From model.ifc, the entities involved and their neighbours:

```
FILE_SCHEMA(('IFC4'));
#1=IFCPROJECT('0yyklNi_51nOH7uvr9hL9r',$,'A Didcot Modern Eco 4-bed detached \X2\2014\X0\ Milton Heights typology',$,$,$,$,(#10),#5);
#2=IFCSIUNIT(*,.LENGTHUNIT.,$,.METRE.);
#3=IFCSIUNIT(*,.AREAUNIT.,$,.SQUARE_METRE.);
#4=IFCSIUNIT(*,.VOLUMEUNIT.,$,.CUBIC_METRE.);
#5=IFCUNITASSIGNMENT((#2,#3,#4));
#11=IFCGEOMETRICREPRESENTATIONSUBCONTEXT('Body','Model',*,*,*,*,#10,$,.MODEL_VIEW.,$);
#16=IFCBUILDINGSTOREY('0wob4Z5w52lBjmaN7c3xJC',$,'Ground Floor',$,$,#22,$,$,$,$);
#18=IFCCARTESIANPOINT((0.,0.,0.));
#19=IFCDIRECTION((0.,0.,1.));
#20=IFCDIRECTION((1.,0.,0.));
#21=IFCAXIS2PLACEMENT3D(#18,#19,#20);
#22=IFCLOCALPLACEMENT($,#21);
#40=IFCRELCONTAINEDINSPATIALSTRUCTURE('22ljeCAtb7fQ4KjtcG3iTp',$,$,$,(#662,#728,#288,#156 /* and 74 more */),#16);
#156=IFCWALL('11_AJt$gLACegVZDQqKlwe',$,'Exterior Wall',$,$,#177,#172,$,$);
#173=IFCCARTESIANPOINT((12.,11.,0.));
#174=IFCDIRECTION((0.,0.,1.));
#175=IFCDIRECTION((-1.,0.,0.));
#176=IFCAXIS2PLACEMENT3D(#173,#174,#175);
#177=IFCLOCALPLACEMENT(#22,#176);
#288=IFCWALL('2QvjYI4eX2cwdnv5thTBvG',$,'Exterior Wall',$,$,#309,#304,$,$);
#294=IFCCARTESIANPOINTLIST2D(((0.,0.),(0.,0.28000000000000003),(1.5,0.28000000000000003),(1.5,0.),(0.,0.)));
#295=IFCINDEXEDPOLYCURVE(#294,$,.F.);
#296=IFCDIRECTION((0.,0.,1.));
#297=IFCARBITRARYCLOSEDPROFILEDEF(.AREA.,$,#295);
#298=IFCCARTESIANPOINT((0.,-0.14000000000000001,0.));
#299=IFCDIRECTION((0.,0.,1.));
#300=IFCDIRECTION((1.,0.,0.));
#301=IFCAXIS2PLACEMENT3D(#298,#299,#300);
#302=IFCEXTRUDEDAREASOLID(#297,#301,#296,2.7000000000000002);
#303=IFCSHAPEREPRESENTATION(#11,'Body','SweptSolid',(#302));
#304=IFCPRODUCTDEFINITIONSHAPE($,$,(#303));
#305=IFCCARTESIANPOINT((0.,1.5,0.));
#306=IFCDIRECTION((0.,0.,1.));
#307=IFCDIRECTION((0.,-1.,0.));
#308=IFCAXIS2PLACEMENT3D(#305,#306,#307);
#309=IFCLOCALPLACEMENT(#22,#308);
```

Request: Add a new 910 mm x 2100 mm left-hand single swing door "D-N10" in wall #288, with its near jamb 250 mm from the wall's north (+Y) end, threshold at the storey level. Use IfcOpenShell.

```python
import numpy as np
import ifcopenshell
import ifcopenshell.api.feature
import ifcopenshell.api.geometry
import ifcopenshell.api.root
import ifcopenshell.api.spatial
import ifcopenshell.geom
import ifcopenshell.util.element
import ifcopenshell.util.placement
import ifcopenshell.util.representation
import ifcopenshell.util.shape
import ifcopenshell.util.unit

model = ifcopenshell.open("model.ifc")
unit_scale = ifcopenshell.util.unit.calculate_unit_scale(model)
settings = ifcopenshell.geom.settings()


def volume(element):
    """Net volume in cubic metres, openings subtracted."""
    shape = ifcopenshell.geom.create_shape(settings, element)
    return ifcopenshell.util.shape.get_volume(shape.geometry)


wall = model.by_id(288)
storey = ifcopenshell.util.element.get_container(wall, ifc_class="IfcBuildingStorey")
context = ifcopenshell.util.representation.get_context(model, "Model", "Body", "MODEL_VIEW")
before = volume(wall)

width, height, from_end, sill = 0.91, 2.1, 0.25, 0.0  # metres

# The wall runs along its own X axis, and the end named is its -X end.
wall_shape = ifcopenshell.geom.create_shape(settings, wall)
x, y, z = ifcopenshell.util.shape.get_vertices(wall_shape.geometry).T
start = x.min() + from_end
face, thickness = float(y.min()), float(y.max() - y.min())
wall_matrix = ifcopenshell.util.placement.get_local_placement(wall.ObjectPlacement)
level = ifcopenshell.util.placement.get_local_placement(storey.ObjectPlacement)[2, 3]


def in_wall(x, y):
    """Placement at x, y metres in the wall's axes, at sill height."""
    matrix = wall_matrix.copy()
    matrix[:, 3] = wall_matrix @ np.array([x / unit_scale, y / unit_scale, 0.0, 1.0])
    matrix[2, 3] = level + sill / unit_scale
    return matrix


# Opening: a box that overshoots both wall faces by 50 mm.
opening = ifcopenshell.api.root.create_entity(model, ifc_class="IfcOpeningElement", predefined_type="OPENING")
box = ifcopenshell.api.geometry.add_wall_representation(
    model, context=context, length=width, height=height, thickness=thickness + 0.1
)
ifcopenshell.api.geometry.assign_representation(model, product=opening, representation=box)
ifcopenshell.api.geometry.edit_object_placement(model, product=opening, matrix=in_wall(start, face - 0.05), is_si=False)
ifcopenshell.api.feature.add_feature(model, feature=opening, element=wall)

door = ifcopenshell.api.root.create_entity(model, ifc_class="IfcDoor", name="D-N10", predefined_type="DOOR")
door.OverallWidth, door.OverallHeight = width / unit_scale, height / unit_scale
door.OperationType = "SINGLE_SWING_LEFT"
body = ifcopenshell.api.geometry.add_door_representation(
    model,
    context=context,
    overall_width=door.OverallWidth,
    overall_height=door.OverallHeight,
    operation_type="SINGLE_SWING_LEFT",
    lining_properties={"LiningDepth": thickness / unit_scale, "ThresholdDepth": thickness / unit_scale},
)
ifcopenshell.api.geometry.assign_representation(model, product=door, representation=body)
ifcopenshell.api.spatial.assign_container(model, products=[door], relating_structure=storey)
ifcopenshell.api.feature.add_filling(model, opening=opening, element=door)

# The lining spans the wall, so the door starts at the wall face.
ifcopenshell.api.geometry.edit_object_placement(model, product=door, matrix=in_wall(start, face), is_si=False)

after = volume(wall)

print(f"wall volume {before:.3f} -> {after:.3f} m3")

model.write("model-out.ifc")
```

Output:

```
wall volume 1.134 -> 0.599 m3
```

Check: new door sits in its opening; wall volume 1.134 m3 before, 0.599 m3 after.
